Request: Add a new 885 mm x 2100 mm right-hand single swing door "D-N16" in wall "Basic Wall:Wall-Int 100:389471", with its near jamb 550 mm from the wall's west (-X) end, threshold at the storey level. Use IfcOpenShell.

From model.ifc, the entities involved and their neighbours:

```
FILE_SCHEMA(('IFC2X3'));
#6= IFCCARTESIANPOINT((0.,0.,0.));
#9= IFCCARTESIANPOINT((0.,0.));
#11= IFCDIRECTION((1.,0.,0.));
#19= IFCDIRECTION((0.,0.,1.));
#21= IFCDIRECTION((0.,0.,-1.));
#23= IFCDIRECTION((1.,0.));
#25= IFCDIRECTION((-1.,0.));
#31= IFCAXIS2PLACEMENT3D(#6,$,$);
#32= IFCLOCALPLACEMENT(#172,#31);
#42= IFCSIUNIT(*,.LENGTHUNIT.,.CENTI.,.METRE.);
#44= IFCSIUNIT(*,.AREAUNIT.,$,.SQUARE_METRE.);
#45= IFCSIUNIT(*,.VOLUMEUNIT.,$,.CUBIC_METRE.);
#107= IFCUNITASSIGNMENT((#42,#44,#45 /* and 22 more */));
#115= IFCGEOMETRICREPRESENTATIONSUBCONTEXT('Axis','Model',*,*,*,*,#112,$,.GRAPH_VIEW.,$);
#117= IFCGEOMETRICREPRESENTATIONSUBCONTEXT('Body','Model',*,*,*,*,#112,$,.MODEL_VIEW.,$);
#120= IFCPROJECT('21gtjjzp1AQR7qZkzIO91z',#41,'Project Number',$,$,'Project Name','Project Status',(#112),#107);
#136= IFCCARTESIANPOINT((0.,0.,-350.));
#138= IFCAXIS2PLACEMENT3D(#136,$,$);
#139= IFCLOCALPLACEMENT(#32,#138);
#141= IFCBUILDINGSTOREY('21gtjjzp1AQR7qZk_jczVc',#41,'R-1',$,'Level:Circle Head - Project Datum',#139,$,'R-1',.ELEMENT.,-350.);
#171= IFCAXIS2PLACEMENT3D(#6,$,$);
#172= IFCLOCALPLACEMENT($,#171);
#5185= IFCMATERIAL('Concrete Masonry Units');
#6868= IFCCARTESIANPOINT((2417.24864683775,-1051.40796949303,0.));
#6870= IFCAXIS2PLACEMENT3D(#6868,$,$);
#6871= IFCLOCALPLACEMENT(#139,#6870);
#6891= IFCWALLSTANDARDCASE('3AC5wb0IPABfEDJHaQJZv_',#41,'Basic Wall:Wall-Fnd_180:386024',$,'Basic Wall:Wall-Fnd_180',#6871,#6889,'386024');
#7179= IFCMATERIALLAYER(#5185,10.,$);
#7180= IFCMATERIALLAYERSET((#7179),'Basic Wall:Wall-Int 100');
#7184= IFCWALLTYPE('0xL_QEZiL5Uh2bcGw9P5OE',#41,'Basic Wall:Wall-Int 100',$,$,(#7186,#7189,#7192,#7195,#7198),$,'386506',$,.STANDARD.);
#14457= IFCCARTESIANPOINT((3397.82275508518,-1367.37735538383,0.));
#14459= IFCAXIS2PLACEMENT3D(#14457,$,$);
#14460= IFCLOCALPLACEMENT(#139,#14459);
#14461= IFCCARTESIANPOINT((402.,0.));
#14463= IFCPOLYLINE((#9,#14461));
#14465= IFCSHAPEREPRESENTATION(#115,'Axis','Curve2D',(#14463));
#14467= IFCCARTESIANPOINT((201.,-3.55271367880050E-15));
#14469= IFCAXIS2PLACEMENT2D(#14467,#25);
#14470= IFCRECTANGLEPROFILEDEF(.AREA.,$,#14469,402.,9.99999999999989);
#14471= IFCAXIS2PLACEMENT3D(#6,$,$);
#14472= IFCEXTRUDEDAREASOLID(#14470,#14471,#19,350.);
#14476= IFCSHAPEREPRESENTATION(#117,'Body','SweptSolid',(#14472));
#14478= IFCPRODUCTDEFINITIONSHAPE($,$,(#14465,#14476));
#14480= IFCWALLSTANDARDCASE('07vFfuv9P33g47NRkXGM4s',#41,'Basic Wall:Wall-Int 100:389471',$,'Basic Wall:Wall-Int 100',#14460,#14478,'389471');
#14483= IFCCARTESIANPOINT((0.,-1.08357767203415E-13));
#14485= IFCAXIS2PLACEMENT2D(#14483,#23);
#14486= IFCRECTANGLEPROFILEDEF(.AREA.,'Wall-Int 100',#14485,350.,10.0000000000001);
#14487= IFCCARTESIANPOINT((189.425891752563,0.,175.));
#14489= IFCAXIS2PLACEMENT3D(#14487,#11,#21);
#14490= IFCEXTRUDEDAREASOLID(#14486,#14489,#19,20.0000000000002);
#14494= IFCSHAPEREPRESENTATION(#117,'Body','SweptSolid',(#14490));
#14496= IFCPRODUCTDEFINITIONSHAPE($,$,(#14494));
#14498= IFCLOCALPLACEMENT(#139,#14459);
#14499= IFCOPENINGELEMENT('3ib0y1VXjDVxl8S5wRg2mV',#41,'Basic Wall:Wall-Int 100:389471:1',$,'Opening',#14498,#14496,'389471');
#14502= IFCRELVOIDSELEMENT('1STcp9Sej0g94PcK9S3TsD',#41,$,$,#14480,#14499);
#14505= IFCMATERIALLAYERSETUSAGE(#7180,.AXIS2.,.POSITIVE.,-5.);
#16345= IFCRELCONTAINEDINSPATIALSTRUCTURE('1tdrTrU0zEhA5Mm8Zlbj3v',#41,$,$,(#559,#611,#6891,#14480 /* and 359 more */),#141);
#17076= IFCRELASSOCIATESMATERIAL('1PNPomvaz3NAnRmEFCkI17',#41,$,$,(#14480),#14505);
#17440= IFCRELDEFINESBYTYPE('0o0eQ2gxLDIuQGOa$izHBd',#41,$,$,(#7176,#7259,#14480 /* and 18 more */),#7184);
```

```python
import numpy as np
import ifcopenshell
import ifcopenshell.api.feature
import ifcopenshell.api.geometry
import ifcopenshell.api.root
import ifcopenshell.api.spatial
import ifcopenshell.api.type
import ifcopenshell.geom
import ifcopenshell.util.element
import ifcopenshell.util.placement
import ifcopenshell.util.representation
import ifcopenshell.util.shape
import ifcopenshell.util.unit

model = ifcopenshell.open("model.ifc")
unit_scale = ifcopenshell.util.unit.calculate_unit_scale(model)
settings = ifcopenshell.geom.settings()


def volume(element):
    """Net volume in cubic metres, openings subtracted."""
    shape = ifcopenshell.geom.create_shape(settings, element)
    return ifcopenshell.util.shape.get_volume(shape.geometry)


wall = model.by_guid("07vFfuv9P33g47NRkXGM4s")
storey = ifcopenshell.util.element.get_container(wall, ifc_class="IfcBuildingStorey")
context = ifcopenshell.util.representation.get_context(model, "Model", "Body", "MODEL_VIEW")
before = volume(wall)

width, height, from_end, sill = 0.885, 2.1, 0.55, 0.0  # metres

# The wall runs along its own X axis, and the end named is its -X end.
wall_shape = ifcopenshell.geom.create_shape(settings, wall)
x, y, z = ifcopenshell.util.shape.get_vertices(wall_shape.geometry).T
start = x.min() + from_end
face, thickness = float(y.min()), float(y.max() - y.min())
wall_matrix = ifcopenshell.util.placement.get_local_placement(wall.ObjectPlacement)
level = ifcopenshell.util.placement.get_local_placement(storey.ObjectPlacement)[2, 3]


def in_wall(x, y):
    """Placement at x, y metres in the wall's axes, at sill height."""
    matrix = wall_matrix.copy()
    matrix[:, 3] = wall_matrix @ np.array([x / unit_scale, y / unit_scale, 0.0, 1.0])
    matrix[2, 3] = level + sill / unit_scale
    return matrix


# Opening: a box that overshoots both wall faces by 50 mm.
opening = ifcopenshell.api.root.create_entity(model, ifc_class="IfcOpeningElement")
box = ifcopenshell.api.geometry.add_wall_representation(
    model, context=context, length=width, height=height, thickness=thickness + 0.1
)
ifcopenshell.api.geometry.assign_representation(model, product=opening, representation=box)
ifcopenshell.api.geometry.edit_object_placement(model, product=opening, matrix=in_wall(start, face - 0.05), is_si=False)
ifcopenshell.api.feature.add_feature(model, feature=opening, element=wall)

door = ifcopenshell.api.root.create_entity(model, ifc_class="IfcDoor", name="D-N16")
door.OverallWidth, door.OverallHeight = width / unit_scale, height / unit_scale
body = ifcopenshell.api.geometry.add_door_representation(
    model,
    context=context,
    overall_width=door.OverallWidth,
    overall_height=door.OverallHeight,
    operation_type="SINGLE_SWING_RIGHT",
    lining_properties={"LiningDepth": thickness / unit_scale, "ThresholdDepth": thickness / unit_scale},
)
ifcopenshell.api.geometry.assign_representation(model, product=door, representation=body)
ifcopenshell.api.spatial.assign_container(model, products=[door], relating_structure=storey)
fills = ifcopenshell.api.feature.add_filling(model, opening=opening, element=door)
fills.OwnerHistory = door.OwnerHistory  # required in IFC2X3

# IFC2X3 keeps the operation on the door style.
style = ifcopenshell.api.root.create_entity(model, ifc_class="IfcDoorStyle", name="D-N16")
style.OperationType, style.ConstructionType = "SINGLE_SWING_RIGHT", "NOTDEFINED"
style.ParameterTakesPrecedence = style.Sizeable = False
ifcopenshell.api.type.assign_type(model, related_objects=[door], relating_type=style)

# The lining spans the wall, so the door starts at the wall face.
ifcopenshell.api.geometry.edit_object_placement(model, product=door, matrix=in_wall(start, face), is_si=False)

after = volume(wall)

print(f"wall volume {before:.3f} -> {after:.3f} m3")

model.write("model_updated.ifc")
```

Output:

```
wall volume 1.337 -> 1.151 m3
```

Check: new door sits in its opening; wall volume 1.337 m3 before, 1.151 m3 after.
